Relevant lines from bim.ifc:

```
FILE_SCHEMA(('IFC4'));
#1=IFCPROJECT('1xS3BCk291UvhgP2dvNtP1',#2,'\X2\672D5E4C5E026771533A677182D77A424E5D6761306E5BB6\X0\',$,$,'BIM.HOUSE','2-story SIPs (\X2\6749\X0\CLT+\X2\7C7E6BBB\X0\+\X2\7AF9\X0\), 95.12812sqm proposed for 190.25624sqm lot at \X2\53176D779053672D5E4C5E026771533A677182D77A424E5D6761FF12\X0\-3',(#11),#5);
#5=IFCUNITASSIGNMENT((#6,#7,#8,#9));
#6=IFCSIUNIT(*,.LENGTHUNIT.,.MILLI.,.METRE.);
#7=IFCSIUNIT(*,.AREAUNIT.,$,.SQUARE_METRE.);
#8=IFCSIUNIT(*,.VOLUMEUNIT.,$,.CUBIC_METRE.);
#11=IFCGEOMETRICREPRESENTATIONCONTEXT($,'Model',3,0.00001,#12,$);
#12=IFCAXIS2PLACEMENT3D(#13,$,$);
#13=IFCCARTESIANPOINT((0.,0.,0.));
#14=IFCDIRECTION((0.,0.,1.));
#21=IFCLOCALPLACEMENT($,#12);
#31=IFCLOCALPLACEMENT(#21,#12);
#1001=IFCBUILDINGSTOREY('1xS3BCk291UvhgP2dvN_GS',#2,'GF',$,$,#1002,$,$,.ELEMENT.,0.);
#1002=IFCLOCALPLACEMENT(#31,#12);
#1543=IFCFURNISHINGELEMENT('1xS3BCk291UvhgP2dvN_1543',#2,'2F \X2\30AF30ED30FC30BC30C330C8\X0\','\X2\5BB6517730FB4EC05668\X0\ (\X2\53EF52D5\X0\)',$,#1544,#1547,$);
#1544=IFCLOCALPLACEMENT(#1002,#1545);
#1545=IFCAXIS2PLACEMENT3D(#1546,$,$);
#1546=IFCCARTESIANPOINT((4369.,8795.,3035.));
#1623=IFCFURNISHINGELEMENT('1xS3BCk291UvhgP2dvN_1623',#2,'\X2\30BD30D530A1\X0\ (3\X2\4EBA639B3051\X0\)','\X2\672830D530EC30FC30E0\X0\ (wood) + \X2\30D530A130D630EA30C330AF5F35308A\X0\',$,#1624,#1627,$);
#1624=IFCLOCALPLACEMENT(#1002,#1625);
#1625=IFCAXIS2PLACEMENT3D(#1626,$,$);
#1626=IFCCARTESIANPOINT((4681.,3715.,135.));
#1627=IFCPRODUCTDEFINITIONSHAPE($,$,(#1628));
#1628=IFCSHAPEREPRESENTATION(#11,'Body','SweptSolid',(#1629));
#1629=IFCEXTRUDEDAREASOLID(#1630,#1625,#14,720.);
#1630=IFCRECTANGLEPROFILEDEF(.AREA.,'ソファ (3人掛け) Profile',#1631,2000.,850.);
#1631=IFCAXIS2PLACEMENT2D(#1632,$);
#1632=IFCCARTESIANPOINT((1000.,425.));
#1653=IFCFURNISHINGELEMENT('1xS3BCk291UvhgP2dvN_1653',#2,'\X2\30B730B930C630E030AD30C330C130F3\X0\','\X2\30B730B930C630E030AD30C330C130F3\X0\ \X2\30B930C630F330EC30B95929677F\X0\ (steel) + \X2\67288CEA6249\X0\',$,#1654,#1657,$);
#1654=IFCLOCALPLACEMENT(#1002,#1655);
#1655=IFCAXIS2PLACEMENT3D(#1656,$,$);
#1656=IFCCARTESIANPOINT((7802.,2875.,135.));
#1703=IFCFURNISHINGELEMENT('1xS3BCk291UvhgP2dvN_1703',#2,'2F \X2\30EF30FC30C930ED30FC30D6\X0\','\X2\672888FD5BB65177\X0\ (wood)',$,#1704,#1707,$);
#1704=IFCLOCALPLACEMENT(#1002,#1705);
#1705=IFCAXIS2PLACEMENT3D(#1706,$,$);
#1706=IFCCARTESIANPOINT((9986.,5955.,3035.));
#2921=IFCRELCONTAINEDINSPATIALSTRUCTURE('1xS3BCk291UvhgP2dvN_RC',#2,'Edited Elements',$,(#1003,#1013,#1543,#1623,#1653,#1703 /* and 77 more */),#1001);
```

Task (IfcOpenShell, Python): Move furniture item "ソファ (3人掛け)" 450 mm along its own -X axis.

```python
import ifcopenshell
import ifcopenshell.api.geometry
import ifcopenshell.util.placement
import ifcopenshell.util.unit

model = ifcopenshell.open("bim.ifc")
unit_scale = ifcopenshell.util.unit.calculate_unit_scale(model)

item = model.by_guid("1xS3BCk291UvhgP2dvN_1623")
matrix = ifcopenshell.util.placement.get_local_placement(item.ObjectPlacement)
matrix[:3, 3] -= matrix[:3, 0] * 0.45 / unit_scale
ifcopenshell.api.geometry.edit_object_placement(model, product=item, matrix=matrix, is_si=False)

print(ifcopenshell.util.placement.get_local_placement(item.ObjectPlacement).round(3) + 0.0)

model.write("bim_v2.ifc")
```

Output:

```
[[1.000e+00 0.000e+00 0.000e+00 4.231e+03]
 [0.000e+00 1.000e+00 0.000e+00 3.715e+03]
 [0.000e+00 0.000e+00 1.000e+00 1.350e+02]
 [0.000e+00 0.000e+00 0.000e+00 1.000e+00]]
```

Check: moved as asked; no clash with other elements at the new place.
